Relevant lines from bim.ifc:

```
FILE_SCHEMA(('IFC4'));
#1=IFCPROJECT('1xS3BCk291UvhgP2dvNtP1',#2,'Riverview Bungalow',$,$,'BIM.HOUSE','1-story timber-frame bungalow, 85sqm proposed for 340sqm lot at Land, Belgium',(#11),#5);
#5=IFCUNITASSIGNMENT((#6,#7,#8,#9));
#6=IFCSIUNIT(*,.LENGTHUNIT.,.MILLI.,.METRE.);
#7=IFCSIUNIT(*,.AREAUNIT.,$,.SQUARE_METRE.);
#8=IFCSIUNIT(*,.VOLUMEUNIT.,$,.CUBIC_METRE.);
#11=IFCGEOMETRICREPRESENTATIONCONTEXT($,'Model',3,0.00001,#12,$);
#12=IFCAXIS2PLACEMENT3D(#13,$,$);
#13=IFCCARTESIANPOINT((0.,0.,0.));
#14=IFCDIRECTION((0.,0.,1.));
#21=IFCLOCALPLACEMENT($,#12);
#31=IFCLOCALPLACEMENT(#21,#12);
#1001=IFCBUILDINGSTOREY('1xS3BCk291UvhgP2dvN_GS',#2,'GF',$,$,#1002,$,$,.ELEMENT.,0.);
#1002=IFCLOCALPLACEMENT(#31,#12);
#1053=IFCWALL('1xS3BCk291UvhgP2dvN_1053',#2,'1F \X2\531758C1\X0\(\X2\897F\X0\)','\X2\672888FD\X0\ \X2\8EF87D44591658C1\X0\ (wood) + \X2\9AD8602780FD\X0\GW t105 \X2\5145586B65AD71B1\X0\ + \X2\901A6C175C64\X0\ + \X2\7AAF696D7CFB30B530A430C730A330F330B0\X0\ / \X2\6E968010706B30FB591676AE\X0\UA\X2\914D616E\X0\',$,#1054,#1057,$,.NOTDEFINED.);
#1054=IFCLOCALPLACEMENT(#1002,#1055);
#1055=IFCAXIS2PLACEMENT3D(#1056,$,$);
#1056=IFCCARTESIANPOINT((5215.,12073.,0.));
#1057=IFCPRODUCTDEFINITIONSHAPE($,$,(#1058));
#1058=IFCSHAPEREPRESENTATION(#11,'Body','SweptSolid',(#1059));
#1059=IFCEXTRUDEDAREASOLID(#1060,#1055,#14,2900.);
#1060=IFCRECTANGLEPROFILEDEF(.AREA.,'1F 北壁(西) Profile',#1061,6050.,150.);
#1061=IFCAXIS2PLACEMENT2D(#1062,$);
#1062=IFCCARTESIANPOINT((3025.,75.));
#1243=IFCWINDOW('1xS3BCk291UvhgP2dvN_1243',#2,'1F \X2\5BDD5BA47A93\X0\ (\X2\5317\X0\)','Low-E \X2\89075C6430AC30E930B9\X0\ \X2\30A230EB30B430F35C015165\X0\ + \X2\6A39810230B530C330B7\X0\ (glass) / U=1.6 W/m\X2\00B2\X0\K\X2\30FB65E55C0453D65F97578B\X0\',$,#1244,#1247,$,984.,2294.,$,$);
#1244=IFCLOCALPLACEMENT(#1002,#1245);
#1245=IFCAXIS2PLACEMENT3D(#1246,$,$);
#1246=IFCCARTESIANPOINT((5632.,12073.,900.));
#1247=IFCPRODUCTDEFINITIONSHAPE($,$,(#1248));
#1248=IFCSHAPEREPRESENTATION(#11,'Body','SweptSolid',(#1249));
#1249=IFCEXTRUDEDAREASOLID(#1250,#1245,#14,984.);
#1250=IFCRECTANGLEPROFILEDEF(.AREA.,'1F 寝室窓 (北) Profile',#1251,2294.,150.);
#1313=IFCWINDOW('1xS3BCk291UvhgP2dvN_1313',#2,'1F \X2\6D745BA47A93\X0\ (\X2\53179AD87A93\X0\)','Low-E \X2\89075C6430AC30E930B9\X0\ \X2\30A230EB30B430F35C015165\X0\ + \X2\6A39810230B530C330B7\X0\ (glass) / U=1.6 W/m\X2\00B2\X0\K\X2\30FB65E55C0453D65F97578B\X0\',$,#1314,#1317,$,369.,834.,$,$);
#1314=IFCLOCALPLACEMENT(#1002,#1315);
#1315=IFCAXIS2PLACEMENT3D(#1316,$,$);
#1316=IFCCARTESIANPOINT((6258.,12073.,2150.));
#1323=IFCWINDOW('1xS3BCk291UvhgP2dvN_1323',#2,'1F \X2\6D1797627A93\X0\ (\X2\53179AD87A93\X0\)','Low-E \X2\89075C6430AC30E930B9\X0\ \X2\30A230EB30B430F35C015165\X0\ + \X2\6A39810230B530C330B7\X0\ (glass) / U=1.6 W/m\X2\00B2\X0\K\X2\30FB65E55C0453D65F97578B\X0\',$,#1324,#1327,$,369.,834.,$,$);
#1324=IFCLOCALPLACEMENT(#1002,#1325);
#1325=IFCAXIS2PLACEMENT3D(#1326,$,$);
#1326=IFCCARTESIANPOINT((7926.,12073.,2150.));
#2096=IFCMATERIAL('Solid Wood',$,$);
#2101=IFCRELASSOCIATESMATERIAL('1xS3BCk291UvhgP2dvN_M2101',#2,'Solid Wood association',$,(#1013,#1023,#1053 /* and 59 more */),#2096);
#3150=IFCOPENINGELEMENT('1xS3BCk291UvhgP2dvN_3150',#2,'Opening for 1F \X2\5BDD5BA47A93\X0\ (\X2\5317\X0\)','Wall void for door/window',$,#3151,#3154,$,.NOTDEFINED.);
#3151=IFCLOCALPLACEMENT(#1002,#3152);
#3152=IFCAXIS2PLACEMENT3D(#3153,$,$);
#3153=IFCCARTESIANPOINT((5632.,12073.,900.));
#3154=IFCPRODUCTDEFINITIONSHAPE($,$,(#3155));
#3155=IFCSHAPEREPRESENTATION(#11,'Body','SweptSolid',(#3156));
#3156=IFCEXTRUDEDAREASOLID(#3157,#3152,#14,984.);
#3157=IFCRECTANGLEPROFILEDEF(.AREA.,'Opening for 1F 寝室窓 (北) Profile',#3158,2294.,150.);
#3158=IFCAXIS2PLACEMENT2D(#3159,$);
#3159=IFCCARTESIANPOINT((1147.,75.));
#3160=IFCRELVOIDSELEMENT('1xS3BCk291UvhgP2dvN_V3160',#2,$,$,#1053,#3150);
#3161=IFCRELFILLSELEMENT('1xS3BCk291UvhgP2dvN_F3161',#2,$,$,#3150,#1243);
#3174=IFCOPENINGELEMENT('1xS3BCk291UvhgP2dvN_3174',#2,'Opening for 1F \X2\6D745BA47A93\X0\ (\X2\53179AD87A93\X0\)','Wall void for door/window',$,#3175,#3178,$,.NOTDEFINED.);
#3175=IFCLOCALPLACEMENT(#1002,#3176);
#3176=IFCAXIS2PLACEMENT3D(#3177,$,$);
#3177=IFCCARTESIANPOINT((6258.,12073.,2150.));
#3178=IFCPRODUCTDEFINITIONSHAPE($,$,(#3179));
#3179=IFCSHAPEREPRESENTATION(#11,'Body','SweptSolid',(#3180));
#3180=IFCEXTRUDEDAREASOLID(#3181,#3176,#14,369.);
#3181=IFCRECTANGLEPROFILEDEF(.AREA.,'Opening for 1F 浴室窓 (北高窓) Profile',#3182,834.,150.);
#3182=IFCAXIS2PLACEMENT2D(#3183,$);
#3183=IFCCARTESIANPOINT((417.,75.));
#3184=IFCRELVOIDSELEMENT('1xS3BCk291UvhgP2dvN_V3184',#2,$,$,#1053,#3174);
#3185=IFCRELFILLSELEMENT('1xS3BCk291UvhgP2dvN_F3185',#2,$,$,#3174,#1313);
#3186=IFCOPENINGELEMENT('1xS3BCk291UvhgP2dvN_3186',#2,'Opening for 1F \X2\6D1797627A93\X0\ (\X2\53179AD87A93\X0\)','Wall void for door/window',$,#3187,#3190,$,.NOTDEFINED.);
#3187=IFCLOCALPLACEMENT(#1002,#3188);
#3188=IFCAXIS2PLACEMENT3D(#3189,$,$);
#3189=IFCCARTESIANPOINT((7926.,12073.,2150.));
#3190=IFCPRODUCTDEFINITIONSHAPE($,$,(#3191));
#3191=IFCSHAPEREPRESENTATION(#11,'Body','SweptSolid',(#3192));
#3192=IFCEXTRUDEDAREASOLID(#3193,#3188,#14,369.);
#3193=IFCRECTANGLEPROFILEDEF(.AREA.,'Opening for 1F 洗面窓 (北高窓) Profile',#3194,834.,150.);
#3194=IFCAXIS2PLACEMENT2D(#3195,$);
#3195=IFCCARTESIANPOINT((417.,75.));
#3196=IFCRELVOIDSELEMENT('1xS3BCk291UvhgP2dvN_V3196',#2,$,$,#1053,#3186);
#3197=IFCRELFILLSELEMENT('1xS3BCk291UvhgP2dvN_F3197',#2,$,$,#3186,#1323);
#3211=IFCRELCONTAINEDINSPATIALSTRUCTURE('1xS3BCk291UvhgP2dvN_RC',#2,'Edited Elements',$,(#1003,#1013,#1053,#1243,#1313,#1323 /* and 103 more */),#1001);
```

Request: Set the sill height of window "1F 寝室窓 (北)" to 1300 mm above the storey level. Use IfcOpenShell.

```python
import numpy as np
import ifcopenshell
import ifcopenshell.api.geometry
import ifcopenshell.geom
import ifcopenshell.util.element
import ifcopenshell.util.placement
import ifcopenshell.util.shape
import ifcopenshell.util.unit

model = ifcopenshell.open("bim.ifc")
unit_scale = ifcopenshell.util.unit.calculate_unit_scale(model)

window = model.by_id(1243)
opening = window.FillsVoids[0].RelatingOpeningElement
storey = ifcopenshell.util.element.get_container(window, ifc_class="IfcBuildingStorey")
level = ifcopenshell.util.placement.get_local_placement(storey.ObjectPlacement)[2, 3]

# The opening's origin need not be at the sill, so measure its lowest point.
shape = ifcopenshell.geom.create_shape(ifcopenshell.geom.settings(), opening)
bottom = ifcopenshell.util.shape.get_shape_bottom_elevation(shape, shape.geometry) / unit_scale
dz = level + 1300.0 - bottom

shift = np.array([0.0, 0.0, dz])
# The window is not placed relative to its opening, so move both.
for product in (opening, window):
    matrix = ifcopenshell.util.placement.get_local_placement(product.ObjectPlacement)
    matrix[:3, 3] += shift
    ifcopenshell.api.geometry.edit_object_placement(model, product=product, matrix=matrix, is_si=False)

print(f"moved by {dz * unit_scale:+.3f} m")

model.write("bim_v2.ifc")
```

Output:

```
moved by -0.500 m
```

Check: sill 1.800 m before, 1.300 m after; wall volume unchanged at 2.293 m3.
